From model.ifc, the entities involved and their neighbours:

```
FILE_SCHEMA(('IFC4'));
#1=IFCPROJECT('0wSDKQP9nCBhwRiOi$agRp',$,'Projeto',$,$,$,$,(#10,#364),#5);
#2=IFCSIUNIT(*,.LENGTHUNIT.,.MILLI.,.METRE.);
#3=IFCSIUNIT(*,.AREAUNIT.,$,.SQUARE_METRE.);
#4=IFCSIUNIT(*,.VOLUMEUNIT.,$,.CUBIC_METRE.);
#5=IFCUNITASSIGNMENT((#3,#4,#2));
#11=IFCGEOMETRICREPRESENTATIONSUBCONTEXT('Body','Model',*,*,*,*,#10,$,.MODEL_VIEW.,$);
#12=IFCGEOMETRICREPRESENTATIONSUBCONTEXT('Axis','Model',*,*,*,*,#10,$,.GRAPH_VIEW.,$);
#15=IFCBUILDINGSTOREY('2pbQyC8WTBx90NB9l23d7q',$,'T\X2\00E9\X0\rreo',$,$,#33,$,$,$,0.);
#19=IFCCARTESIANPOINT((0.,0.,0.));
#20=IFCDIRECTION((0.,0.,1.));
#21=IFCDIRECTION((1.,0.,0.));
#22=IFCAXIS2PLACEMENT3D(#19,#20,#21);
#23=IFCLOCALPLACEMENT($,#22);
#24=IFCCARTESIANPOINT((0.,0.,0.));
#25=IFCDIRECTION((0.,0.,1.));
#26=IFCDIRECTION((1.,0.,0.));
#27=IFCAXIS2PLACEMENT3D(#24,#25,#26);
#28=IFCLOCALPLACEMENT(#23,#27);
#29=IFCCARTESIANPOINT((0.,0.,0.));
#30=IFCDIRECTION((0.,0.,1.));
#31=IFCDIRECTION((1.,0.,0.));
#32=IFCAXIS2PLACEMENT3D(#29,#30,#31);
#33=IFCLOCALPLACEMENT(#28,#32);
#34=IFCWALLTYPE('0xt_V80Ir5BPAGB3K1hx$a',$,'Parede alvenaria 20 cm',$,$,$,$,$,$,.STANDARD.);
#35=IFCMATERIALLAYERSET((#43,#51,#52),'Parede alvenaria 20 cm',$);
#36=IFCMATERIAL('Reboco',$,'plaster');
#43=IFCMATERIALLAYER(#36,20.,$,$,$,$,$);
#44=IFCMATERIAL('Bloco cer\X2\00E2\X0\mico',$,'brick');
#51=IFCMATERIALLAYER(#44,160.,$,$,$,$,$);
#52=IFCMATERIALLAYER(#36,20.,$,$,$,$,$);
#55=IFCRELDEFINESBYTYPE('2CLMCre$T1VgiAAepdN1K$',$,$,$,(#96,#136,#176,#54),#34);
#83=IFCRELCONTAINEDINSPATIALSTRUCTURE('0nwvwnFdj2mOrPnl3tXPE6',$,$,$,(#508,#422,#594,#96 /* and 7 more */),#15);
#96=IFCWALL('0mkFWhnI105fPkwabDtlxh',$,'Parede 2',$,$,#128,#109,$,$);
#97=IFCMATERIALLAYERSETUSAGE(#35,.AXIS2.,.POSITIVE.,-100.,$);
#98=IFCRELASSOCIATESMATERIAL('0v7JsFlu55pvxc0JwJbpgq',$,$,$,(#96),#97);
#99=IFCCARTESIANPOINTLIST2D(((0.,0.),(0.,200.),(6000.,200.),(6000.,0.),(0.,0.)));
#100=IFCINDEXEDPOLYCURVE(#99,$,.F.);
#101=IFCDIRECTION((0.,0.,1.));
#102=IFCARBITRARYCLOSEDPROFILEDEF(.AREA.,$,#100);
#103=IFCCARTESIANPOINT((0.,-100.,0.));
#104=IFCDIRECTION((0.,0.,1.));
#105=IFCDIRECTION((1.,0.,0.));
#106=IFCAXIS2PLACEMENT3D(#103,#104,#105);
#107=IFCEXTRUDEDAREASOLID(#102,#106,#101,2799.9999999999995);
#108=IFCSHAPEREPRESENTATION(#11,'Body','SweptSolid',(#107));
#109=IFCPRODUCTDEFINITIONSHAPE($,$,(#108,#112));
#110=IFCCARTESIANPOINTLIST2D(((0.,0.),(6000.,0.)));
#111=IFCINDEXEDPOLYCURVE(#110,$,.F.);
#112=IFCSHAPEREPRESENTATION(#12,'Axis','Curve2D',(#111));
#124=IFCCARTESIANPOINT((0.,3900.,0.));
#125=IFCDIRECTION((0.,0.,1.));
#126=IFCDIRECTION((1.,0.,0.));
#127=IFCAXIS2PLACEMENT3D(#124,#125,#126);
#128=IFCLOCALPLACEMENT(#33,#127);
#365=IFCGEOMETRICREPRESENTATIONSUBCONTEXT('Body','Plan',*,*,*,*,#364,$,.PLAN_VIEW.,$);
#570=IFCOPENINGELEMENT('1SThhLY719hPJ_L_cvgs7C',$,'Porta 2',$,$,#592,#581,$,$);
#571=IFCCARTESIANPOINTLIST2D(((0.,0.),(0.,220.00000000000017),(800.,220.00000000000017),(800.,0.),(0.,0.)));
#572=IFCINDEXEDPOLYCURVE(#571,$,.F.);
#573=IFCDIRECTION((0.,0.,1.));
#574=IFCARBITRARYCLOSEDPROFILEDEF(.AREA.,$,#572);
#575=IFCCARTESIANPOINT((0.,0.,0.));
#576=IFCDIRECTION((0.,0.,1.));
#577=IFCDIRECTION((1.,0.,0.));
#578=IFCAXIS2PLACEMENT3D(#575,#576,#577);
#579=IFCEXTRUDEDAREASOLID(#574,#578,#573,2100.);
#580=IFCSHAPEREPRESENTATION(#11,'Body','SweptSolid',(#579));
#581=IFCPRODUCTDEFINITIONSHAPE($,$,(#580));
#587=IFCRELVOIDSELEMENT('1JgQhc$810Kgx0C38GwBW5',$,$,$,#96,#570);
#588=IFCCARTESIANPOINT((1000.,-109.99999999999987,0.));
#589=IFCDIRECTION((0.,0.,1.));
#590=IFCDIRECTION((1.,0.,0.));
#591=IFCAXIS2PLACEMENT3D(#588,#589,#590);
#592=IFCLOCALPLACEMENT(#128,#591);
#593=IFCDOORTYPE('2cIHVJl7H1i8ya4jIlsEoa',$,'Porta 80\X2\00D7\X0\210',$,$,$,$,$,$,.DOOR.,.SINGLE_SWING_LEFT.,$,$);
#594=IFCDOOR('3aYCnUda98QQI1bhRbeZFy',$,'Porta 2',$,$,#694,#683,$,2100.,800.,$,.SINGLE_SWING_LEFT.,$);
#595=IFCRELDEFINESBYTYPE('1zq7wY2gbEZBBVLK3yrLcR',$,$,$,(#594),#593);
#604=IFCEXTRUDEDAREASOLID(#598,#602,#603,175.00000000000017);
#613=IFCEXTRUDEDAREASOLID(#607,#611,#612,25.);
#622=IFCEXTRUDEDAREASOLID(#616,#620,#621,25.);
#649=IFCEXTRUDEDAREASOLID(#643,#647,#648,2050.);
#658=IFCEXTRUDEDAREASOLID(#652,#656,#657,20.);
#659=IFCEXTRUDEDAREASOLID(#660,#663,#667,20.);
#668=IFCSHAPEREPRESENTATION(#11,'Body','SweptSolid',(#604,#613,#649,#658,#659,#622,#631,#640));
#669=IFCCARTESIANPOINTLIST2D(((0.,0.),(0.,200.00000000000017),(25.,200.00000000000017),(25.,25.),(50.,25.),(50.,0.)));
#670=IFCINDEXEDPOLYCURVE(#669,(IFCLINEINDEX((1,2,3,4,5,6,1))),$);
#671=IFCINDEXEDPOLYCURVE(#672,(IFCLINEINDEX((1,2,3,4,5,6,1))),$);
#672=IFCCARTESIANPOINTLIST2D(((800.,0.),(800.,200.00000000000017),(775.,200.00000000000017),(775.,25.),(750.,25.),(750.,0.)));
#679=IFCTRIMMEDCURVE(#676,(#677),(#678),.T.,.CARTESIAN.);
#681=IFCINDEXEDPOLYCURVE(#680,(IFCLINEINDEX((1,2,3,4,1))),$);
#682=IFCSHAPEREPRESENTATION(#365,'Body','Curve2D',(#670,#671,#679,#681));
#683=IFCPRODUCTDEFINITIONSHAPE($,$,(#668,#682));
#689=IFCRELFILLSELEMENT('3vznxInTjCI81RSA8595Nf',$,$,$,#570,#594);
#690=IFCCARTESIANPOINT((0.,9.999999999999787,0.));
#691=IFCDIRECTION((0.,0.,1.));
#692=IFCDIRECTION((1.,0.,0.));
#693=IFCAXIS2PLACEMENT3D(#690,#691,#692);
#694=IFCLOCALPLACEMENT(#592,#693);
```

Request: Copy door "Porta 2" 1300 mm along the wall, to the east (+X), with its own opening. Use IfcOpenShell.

```python
import ifcopenshell
import ifcopenshell.api.feature
import ifcopenshell.api.geometry
import ifcopenshell.api.root
import ifcopenshell.geom
import ifcopenshell.util.element
import ifcopenshell.util.placement
import ifcopenshell.util.shape
import ifcopenshell.util.unit

model = ifcopenshell.open("model.ifc")
unit_scale = ifcopenshell.util.unit.calculate_unit_scale(model)
settings = ifcopenshell.geom.settings()


def volume(element):
    """Net volume in cubic metres, openings subtracted."""
    shape = ifcopenshell.geom.create_shape(settings, element)
    return ifcopenshell.util.shape.get_volume(shape.geometry)


door = model.by_guid("3aYCnUda98QQI1bhRbeZFy")
opening = door.FillsVoids[0].RelatingOpeningElement
wall = opening.VoidsElements[0].RelatingBuildingElement
before = volume(wall)
shift = ifcopenshell.util.placement.get_local_placement(wall.ObjectPlacement)[:3, 0] * 1.3 / unit_scale

# copy_class copies the void relationship, type, container and properties, but no geometry.
new_opening = ifcopenshell.api.root.copy_class(model, product=opening)
new_opening.Representation = ifcopenshell.util.element.copy_deep(
    model, opening.Representation, exclude=["IfcGeometricRepresentationContext", "IfcRepresentationMap"]
)
new_door = ifcopenshell.api.root.copy_class(model, product=door)
new_door.Representation = ifcopenshell.util.element.copy_deep(
    model, door.Representation, exclude=["IfcGeometricRepresentationContext", "IfcRepresentationMap"]
)
ifcopenshell.api.feature.add_filling(model, opening=new_opening, element=new_door)

for old, new in ((opening, new_opening), (door, new_door)):
    matrix = ifcopenshell.util.placement.get_local_placement(old.ObjectPlacement)
    matrix[:3, 3] += shift
    ifcopenshell.api.geometry.edit_object_placement(model, product=new, matrix=matrix, is_si=False)

after = volume(wall)

print(f"wall volume {before:.3f} -> {after:.3f} m3")

model.write("model_edited.ifc")
```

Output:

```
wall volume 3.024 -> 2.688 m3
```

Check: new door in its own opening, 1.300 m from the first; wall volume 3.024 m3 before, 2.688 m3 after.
